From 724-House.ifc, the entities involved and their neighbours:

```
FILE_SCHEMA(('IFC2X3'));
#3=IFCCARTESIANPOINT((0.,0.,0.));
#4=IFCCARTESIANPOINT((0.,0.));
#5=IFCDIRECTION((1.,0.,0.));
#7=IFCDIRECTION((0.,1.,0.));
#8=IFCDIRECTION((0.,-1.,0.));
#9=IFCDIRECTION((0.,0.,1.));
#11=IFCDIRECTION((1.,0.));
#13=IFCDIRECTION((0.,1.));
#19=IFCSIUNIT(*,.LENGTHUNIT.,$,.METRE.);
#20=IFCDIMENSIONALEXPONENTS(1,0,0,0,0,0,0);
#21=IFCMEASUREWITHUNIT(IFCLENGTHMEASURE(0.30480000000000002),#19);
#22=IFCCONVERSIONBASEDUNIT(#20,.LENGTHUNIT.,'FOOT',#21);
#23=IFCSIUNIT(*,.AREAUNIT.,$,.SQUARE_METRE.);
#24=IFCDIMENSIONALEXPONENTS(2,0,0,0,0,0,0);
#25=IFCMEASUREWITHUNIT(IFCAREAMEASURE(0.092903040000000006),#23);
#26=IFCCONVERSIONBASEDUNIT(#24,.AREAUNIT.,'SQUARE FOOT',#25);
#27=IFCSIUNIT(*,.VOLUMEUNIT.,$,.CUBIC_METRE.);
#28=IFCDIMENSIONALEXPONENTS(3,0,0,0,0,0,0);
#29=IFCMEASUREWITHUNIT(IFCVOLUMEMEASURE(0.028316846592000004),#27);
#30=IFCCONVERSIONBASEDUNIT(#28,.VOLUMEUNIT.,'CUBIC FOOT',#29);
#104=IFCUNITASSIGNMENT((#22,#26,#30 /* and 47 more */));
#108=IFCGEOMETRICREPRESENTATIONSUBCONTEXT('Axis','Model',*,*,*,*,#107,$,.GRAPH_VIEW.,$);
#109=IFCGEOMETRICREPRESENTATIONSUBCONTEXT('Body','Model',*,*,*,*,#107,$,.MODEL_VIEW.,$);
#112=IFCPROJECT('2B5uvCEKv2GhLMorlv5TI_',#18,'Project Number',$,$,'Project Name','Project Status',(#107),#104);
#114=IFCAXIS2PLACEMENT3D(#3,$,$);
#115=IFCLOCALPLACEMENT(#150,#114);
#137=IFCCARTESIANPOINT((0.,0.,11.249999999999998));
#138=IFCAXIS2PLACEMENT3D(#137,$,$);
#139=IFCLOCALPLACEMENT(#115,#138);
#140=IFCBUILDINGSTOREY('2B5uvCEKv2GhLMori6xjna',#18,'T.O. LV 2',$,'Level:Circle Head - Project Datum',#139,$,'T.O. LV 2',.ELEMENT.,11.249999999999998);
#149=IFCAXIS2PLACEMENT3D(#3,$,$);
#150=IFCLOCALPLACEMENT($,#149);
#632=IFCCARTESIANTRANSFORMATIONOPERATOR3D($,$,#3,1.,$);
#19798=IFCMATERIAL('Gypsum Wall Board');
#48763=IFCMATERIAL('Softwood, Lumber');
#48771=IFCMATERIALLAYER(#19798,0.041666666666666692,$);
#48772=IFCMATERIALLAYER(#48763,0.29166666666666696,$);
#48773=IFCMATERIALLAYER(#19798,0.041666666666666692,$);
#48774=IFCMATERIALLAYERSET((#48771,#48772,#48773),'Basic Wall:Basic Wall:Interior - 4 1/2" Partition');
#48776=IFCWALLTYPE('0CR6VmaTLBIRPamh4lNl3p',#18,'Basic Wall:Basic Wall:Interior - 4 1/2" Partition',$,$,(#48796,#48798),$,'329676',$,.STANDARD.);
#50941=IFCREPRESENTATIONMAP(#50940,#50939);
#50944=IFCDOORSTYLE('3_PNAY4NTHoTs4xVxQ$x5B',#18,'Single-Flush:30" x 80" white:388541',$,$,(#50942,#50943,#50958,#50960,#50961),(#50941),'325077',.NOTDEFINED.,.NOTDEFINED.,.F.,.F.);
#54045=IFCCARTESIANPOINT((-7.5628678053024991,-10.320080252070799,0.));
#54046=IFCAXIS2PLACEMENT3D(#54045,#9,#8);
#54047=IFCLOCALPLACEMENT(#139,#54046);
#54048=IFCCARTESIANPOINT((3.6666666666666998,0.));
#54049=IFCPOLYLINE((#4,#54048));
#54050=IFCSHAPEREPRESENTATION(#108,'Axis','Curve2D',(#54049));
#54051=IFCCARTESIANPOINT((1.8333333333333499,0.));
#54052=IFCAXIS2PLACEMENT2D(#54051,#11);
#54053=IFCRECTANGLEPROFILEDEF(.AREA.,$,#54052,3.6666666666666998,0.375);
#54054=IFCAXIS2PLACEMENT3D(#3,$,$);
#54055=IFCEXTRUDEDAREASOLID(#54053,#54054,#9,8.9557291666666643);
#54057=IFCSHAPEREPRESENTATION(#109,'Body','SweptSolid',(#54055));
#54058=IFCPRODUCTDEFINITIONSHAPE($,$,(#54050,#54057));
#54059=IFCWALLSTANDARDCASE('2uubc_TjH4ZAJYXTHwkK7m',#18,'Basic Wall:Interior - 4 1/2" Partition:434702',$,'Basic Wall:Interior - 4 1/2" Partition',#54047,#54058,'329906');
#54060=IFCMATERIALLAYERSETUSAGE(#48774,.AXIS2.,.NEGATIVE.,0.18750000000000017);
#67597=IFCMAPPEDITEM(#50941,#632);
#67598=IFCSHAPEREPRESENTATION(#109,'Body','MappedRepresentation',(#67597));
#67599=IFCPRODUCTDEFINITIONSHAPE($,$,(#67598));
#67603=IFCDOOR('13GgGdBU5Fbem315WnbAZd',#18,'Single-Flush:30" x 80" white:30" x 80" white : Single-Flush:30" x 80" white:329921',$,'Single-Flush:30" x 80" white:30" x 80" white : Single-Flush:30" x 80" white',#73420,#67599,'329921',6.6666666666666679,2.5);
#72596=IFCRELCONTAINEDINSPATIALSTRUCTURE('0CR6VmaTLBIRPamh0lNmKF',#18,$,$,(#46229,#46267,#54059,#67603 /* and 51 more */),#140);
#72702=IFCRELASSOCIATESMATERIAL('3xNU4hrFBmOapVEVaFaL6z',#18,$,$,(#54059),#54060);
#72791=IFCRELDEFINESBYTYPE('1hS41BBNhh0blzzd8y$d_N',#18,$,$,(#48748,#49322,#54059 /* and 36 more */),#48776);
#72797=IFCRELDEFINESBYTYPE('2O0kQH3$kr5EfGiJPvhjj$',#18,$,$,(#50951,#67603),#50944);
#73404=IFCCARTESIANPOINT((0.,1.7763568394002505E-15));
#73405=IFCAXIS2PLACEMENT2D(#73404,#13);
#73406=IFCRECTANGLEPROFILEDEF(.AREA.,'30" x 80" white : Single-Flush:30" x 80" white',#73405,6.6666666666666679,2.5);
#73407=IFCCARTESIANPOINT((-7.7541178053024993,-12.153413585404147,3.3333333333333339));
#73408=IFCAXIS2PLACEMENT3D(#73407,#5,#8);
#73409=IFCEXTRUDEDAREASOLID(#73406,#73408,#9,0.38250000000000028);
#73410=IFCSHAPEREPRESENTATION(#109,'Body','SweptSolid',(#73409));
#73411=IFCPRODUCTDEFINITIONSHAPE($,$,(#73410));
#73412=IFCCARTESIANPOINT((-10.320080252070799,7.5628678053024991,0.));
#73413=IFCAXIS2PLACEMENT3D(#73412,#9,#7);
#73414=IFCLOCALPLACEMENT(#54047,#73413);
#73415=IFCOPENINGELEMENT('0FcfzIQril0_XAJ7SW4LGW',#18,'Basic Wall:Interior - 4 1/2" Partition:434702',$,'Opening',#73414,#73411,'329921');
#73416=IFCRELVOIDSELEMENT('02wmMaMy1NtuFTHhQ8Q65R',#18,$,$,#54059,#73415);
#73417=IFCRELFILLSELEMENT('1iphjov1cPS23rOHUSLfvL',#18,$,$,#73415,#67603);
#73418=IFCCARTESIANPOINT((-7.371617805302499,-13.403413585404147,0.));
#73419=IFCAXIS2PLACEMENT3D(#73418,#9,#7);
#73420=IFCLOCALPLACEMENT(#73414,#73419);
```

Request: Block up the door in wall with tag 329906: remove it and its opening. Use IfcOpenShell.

```python
import ifcopenshell
import ifcopenshell.api.feature
import ifcopenshell.api.root
import ifcopenshell.geom
import ifcopenshell.util.shape

model = ifcopenshell.open("724-House.ifc")
settings = ifcopenshell.geom.settings()


def volume(element):
    """Net volume in cubic metres, openings subtracted."""
    shape = ifcopenshell.geom.create_shape(settings, element)
    return ifcopenshell.util.shape.get_volume(shape.geometry)


door = model.by_guid("13GgGdBU5Fbem315WnbAZd")
opening = door.FillsVoids[0].RelatingOpeningElement
wall = opening.VoidsElements[0].RelatingBuildingElement
before = volume(wall)

ifcopenshell.api.root.remove_product(model, product=door)
ifcopenshell.api.feature.remove_feature(model, feature=opening)

after = volume(wall)

print(f"wall volume {before:.3f} -> {after:.3f} m3")

model.write("724-House_updated.ifc")
```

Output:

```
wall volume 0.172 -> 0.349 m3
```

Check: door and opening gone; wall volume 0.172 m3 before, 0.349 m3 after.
